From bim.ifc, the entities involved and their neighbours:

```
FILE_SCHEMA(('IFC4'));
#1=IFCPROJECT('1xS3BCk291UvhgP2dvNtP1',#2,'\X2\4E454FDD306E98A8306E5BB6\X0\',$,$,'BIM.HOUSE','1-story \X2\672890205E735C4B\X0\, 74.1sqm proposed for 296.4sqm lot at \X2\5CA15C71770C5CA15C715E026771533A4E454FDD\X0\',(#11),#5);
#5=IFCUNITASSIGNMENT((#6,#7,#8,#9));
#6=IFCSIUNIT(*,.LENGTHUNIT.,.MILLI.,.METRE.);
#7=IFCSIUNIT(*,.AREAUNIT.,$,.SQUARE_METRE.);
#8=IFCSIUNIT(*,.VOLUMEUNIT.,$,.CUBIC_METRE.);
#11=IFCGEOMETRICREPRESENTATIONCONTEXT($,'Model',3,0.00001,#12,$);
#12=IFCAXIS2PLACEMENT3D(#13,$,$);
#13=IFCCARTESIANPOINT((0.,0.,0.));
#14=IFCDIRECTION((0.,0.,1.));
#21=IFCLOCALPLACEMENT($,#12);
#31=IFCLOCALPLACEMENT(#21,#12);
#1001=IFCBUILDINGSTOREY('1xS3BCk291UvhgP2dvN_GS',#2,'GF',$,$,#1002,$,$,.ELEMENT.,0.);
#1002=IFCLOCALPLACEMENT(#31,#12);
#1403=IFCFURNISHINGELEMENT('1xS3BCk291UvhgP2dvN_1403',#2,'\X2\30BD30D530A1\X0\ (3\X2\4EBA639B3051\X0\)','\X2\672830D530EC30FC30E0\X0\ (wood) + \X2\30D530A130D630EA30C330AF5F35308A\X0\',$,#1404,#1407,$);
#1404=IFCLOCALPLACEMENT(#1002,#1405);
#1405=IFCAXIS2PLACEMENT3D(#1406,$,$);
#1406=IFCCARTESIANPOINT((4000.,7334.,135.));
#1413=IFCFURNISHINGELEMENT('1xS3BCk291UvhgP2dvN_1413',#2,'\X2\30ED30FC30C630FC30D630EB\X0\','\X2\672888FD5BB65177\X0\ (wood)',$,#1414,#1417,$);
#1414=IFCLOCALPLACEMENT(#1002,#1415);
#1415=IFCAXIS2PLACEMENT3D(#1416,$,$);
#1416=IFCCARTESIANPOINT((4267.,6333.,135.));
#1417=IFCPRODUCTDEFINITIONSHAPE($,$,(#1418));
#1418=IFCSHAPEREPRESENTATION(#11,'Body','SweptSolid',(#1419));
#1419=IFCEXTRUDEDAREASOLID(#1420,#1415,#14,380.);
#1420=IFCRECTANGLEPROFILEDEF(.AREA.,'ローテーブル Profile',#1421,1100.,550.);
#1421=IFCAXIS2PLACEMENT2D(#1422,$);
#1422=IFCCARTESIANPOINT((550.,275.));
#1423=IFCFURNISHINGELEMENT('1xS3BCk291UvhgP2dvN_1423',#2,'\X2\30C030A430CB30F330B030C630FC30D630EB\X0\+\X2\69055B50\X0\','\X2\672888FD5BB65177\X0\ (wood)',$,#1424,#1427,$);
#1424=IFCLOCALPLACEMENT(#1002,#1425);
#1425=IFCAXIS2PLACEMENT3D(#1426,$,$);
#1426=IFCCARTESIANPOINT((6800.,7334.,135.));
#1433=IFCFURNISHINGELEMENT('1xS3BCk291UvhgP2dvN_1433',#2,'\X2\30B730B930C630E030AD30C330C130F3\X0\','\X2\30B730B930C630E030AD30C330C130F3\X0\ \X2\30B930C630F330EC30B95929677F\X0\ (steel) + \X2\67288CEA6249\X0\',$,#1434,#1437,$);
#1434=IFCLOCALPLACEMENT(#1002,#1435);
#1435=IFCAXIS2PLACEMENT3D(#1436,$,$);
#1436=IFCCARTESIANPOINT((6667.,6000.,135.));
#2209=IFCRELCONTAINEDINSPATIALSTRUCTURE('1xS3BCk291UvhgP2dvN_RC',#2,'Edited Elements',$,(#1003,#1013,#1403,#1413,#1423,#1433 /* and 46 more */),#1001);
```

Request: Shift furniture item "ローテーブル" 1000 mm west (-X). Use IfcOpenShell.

```python
import ifcopenshell
import ifcopenshell.api.geometry
import ifcopenshell.util.placement
import ifcopenshell.util.unit

model = ifcopenshell.open("bim.ifc")
unit_scale = ifcopenshell.util.unit.calculate_unit_scale(model)

item = model.by_id(1413)
matrix = ifcopenshell.util.placement.get_local_placement(item.ObjectPlacement)
matrix[0, 3] -= 1 / unit_scale
ifcopenshell.api.geometry.edit_object_placement(model, product=item, matrix=matrix, is_si=False)

print(ifcopenshell.util.placement.get_local_placement(item.ObjectPlacement).round(3) + 0.0)

model.write("bim_updated.ifc")
```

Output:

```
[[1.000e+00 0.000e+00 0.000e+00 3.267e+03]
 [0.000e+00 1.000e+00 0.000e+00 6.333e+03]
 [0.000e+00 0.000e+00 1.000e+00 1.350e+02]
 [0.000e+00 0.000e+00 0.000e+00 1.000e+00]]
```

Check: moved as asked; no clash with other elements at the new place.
